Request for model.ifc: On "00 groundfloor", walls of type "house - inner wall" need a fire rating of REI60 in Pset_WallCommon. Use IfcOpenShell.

First a look at what the model holds.

```python
import ifcopenshell
import ifcopenshell.util.element

model = ifcopenshell.open("model.ifc")
print(model.schema)
storey = next(s for s in model.by_type("IfcBuildingStorey") if s.Name == "00 groundfloor")
walls = [e for e in ifcopenshell.util.element.get_decomposition(storey) if e.is_a("IfcWall")]
seen = {}
for e in walls:
    element_type = ifcopenshell.util.element.get_type(e)
    key = (element_type.Name if element_type != e and element_type else None, ifcopenshell.util.element.get_pset(e, "Pset_WallCommon", "FireRating"))
    seen[key] = seen.get(key, 0) + 1
for (name, value), count in sorted(seen.items(), key=str):
    print(count, "x", name, "|", value)
```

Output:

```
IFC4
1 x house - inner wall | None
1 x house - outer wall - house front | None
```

```python
import ifcopenshell
import ifcopenshell.api.pset
import ifcopenshell.util.element

model = ifcopenshell.open("model.ifc")

storey = next(s for s in model.by_type("IfcBuildingStorey") if s.Name == "00 groundfloor")
walls = [e for e in ifcopenshell.util.element.get_decomposition(storey) if e.is_a("IfcWall")]

count = 0
for e in walls:
    element_type = ifcopenshell.util.element.get_type(e)
    if element_type in (None, e) or element_type.Name != "house - inner wall":
        continue
    # add_pset returns the element's existing set when there is one.
    pset = ifcopenshell.api.pset.add_pset(model, product=e, name="Pset_WallCommon")
    ifcopenshell.api.pset.edit_pset(model, pset=pset, properties={"FireRating": "REI60"})
    count += 1

print(count, "walls updated")

model.write("model_rev.ifc")
```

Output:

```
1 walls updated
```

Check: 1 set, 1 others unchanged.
